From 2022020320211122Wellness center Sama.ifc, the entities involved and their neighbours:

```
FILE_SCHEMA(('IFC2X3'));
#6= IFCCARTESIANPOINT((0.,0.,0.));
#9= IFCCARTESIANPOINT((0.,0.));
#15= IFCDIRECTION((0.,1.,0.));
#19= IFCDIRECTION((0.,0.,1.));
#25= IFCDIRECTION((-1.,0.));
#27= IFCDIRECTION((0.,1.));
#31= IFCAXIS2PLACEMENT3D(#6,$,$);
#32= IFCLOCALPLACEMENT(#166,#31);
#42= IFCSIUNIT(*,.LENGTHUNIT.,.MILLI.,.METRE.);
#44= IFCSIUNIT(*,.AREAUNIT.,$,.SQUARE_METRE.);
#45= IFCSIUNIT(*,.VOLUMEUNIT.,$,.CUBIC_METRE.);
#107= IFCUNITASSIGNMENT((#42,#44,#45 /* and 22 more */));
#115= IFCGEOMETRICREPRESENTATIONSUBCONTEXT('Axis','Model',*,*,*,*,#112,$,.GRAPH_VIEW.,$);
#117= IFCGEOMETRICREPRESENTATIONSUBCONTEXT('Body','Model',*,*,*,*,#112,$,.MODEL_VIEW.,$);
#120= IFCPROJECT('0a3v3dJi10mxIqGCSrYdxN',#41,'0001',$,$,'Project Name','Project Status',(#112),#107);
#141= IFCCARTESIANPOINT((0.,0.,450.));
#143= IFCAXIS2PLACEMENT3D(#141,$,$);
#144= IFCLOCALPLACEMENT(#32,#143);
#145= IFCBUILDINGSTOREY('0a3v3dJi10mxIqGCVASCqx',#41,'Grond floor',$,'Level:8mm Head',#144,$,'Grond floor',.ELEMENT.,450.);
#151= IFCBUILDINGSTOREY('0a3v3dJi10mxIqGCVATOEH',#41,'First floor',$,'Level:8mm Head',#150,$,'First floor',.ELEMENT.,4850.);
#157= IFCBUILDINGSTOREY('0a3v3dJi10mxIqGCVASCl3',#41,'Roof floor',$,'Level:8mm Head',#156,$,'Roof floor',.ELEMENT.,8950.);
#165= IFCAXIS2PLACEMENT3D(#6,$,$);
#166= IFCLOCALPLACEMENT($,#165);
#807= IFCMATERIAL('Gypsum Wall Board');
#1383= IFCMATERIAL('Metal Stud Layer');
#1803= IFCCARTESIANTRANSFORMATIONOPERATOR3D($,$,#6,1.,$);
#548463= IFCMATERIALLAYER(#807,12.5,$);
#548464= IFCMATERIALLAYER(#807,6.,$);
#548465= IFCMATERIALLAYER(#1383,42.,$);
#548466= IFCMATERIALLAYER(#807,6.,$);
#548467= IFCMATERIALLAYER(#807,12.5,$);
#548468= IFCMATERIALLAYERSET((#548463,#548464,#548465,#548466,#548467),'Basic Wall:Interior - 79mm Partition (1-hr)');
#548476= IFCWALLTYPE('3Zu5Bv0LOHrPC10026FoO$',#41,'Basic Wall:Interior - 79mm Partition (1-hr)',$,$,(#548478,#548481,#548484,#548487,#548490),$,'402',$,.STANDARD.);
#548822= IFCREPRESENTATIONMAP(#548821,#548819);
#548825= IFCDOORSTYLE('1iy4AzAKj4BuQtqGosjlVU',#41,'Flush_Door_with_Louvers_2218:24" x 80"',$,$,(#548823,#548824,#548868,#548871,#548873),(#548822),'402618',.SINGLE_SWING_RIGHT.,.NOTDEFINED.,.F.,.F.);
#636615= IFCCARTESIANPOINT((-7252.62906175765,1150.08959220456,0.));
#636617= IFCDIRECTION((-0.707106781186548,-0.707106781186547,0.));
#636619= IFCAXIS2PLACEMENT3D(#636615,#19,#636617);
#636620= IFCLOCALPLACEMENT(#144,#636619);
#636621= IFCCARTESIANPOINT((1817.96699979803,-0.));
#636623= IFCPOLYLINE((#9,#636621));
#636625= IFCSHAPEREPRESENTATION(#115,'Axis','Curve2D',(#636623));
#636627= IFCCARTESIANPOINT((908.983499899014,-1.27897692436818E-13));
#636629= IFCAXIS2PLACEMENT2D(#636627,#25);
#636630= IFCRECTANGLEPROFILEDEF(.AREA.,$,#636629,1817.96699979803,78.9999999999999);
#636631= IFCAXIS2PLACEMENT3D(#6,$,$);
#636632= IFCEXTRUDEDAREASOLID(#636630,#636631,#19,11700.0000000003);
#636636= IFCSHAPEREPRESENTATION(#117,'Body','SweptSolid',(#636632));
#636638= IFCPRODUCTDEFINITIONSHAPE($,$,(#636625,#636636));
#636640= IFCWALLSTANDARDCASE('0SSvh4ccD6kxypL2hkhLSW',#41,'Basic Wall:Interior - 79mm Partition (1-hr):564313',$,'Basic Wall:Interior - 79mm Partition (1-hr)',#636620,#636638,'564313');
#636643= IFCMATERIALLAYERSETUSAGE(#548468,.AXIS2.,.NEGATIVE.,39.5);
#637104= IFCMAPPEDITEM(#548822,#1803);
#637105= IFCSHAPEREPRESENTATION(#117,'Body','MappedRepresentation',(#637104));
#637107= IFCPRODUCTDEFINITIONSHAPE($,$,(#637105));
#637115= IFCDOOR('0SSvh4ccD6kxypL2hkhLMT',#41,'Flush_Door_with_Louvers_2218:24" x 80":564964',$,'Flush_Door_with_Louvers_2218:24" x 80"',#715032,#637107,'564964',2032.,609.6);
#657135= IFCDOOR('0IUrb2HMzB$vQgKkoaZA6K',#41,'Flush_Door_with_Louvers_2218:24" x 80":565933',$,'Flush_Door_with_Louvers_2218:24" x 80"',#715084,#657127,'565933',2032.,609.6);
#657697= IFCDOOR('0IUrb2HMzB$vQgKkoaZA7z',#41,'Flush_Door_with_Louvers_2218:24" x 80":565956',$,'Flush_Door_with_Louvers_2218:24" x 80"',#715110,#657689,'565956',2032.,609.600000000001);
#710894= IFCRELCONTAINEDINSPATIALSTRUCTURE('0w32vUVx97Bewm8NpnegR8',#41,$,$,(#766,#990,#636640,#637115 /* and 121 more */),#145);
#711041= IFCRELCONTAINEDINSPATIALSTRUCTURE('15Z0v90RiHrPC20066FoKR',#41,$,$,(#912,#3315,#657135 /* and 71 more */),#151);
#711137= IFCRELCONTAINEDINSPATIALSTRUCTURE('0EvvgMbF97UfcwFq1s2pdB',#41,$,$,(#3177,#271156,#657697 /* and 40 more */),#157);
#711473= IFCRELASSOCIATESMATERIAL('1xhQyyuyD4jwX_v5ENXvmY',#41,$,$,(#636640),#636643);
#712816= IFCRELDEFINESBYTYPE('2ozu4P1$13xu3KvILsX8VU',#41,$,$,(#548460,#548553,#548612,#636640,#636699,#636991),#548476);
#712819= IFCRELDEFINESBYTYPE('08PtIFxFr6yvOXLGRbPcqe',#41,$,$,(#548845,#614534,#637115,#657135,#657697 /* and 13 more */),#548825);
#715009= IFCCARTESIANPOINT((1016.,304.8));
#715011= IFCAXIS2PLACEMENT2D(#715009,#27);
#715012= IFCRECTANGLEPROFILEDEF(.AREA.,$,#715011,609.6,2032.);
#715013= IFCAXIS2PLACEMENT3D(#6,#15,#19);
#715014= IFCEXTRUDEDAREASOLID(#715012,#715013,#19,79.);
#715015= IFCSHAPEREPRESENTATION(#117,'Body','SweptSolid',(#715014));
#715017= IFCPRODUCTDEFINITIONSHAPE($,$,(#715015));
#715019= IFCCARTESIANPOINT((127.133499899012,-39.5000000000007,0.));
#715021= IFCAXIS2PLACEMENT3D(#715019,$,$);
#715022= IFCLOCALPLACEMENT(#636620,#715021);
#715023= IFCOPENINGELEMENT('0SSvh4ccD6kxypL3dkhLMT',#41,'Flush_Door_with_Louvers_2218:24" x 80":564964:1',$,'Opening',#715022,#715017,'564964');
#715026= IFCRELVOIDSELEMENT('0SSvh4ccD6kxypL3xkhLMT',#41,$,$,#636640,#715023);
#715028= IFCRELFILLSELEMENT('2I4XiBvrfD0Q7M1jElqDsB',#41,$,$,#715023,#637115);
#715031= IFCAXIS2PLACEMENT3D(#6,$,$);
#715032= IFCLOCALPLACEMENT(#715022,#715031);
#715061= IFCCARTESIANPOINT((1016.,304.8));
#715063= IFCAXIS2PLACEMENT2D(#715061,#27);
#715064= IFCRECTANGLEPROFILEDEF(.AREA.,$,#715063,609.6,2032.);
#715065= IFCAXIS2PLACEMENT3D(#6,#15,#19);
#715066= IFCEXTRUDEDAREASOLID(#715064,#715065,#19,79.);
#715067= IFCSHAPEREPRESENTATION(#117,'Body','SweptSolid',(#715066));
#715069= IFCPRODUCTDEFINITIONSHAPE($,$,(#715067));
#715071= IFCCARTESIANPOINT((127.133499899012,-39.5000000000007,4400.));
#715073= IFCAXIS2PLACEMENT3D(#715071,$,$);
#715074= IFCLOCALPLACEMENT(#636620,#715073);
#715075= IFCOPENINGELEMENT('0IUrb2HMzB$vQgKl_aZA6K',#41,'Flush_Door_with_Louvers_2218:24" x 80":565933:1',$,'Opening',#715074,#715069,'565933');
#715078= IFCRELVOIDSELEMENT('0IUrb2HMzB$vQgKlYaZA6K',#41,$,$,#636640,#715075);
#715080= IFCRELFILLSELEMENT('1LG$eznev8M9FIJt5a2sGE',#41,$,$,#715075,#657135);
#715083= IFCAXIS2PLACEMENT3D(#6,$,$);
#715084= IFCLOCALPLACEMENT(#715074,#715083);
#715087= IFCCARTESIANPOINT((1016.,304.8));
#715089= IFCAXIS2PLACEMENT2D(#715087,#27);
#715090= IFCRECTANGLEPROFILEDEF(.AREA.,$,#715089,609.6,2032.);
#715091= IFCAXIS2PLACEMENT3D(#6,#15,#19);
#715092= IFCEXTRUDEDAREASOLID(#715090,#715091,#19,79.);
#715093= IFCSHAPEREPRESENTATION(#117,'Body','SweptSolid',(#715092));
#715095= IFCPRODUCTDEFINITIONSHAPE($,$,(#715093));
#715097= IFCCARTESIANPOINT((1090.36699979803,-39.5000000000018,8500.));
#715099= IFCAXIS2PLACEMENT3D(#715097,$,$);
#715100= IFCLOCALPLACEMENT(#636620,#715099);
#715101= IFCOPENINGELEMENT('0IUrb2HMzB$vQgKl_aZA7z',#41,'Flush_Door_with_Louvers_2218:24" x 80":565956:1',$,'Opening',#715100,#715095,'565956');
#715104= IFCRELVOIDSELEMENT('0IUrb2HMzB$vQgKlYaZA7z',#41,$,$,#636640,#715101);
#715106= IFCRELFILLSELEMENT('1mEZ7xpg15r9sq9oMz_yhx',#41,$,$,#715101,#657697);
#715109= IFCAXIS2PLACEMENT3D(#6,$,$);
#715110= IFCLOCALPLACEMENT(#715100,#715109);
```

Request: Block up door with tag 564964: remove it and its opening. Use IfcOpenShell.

```python
import ifcopenshell
import ifcopenshell.api.feature
import ifcopenshell.api.root
import ifcopenshell.geom
import ifcopenshell.util.shape

model = ifcopenshell.open("2022020320211122Wellness center Sama.ifc")
settings = ifcopenshell.geom.settings()


def volume(element):
    """Net volume in cubic metres, openings subtracted."""
    shape = ifcopenshell.geom.create_shape(settings, element)
    return ifcopenshell.util.shape.get_volume(shape.geometry)


door = model.by_guid("0SSvh4ccD6kxypL2hkhLMT")
opening = door.FillsVoids[0].RelatingOpeningElement
wall = opening.VoidsElements[0].RelatingBuildingElement
before = volume(wall)

ifcopenshell.api.root.remove_product(model, product=door)
ifcopenshell.api.feature.remove_feature(model, feature=opening)

after = volume(wall)

print(f"wall volume {before:.3f} -> {after:.3f} m3")

model.write("2022020320211122Wellness center Sama_rev.ifc")
```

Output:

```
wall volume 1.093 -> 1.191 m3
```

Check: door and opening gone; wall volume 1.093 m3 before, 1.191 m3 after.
